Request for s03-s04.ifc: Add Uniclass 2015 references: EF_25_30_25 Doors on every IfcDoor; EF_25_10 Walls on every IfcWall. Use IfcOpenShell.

First a look at what the model holds.

```python
import ifcopenshell

model = ifcopenshell.open("s03-s04.ifc")
print(model.schema)
print("classifications:", [c.Name for c in model.by_type("IfcClassification")])
for ifc_class in ("IfcDoor", "IfcRoof", "IfcStair", "IfcWall", "IfcWindow"):
    print(ifc_class, len(model.by_type(ifc_class)))
```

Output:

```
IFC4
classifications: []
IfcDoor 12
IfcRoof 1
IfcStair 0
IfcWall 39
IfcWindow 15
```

```python
import ifcopenshell
import ifcopenshell.api.classification

model = ifcopenshell.open("s03-s04.ifc")

system = ifcopenshell.api.classification.add_classification(model, classification="Uniclass 2015")

codes = {
    "IfcDoor": ("EF_25_30_25", "Doors"),
    "IfcWall": ("EF_25_10", "Walls"),
}
for ifc_class, (code, name) in codes.items():
    products = model.by_type(ifc_class)
    ifcopenshell.api.classification.add_reference(
        model, products=products, classification=system, identification=code, name=name
    )
    print(code, len(products))

model.write("s03-s04_v2.ifc")
```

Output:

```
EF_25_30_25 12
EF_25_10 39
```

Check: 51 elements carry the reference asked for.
